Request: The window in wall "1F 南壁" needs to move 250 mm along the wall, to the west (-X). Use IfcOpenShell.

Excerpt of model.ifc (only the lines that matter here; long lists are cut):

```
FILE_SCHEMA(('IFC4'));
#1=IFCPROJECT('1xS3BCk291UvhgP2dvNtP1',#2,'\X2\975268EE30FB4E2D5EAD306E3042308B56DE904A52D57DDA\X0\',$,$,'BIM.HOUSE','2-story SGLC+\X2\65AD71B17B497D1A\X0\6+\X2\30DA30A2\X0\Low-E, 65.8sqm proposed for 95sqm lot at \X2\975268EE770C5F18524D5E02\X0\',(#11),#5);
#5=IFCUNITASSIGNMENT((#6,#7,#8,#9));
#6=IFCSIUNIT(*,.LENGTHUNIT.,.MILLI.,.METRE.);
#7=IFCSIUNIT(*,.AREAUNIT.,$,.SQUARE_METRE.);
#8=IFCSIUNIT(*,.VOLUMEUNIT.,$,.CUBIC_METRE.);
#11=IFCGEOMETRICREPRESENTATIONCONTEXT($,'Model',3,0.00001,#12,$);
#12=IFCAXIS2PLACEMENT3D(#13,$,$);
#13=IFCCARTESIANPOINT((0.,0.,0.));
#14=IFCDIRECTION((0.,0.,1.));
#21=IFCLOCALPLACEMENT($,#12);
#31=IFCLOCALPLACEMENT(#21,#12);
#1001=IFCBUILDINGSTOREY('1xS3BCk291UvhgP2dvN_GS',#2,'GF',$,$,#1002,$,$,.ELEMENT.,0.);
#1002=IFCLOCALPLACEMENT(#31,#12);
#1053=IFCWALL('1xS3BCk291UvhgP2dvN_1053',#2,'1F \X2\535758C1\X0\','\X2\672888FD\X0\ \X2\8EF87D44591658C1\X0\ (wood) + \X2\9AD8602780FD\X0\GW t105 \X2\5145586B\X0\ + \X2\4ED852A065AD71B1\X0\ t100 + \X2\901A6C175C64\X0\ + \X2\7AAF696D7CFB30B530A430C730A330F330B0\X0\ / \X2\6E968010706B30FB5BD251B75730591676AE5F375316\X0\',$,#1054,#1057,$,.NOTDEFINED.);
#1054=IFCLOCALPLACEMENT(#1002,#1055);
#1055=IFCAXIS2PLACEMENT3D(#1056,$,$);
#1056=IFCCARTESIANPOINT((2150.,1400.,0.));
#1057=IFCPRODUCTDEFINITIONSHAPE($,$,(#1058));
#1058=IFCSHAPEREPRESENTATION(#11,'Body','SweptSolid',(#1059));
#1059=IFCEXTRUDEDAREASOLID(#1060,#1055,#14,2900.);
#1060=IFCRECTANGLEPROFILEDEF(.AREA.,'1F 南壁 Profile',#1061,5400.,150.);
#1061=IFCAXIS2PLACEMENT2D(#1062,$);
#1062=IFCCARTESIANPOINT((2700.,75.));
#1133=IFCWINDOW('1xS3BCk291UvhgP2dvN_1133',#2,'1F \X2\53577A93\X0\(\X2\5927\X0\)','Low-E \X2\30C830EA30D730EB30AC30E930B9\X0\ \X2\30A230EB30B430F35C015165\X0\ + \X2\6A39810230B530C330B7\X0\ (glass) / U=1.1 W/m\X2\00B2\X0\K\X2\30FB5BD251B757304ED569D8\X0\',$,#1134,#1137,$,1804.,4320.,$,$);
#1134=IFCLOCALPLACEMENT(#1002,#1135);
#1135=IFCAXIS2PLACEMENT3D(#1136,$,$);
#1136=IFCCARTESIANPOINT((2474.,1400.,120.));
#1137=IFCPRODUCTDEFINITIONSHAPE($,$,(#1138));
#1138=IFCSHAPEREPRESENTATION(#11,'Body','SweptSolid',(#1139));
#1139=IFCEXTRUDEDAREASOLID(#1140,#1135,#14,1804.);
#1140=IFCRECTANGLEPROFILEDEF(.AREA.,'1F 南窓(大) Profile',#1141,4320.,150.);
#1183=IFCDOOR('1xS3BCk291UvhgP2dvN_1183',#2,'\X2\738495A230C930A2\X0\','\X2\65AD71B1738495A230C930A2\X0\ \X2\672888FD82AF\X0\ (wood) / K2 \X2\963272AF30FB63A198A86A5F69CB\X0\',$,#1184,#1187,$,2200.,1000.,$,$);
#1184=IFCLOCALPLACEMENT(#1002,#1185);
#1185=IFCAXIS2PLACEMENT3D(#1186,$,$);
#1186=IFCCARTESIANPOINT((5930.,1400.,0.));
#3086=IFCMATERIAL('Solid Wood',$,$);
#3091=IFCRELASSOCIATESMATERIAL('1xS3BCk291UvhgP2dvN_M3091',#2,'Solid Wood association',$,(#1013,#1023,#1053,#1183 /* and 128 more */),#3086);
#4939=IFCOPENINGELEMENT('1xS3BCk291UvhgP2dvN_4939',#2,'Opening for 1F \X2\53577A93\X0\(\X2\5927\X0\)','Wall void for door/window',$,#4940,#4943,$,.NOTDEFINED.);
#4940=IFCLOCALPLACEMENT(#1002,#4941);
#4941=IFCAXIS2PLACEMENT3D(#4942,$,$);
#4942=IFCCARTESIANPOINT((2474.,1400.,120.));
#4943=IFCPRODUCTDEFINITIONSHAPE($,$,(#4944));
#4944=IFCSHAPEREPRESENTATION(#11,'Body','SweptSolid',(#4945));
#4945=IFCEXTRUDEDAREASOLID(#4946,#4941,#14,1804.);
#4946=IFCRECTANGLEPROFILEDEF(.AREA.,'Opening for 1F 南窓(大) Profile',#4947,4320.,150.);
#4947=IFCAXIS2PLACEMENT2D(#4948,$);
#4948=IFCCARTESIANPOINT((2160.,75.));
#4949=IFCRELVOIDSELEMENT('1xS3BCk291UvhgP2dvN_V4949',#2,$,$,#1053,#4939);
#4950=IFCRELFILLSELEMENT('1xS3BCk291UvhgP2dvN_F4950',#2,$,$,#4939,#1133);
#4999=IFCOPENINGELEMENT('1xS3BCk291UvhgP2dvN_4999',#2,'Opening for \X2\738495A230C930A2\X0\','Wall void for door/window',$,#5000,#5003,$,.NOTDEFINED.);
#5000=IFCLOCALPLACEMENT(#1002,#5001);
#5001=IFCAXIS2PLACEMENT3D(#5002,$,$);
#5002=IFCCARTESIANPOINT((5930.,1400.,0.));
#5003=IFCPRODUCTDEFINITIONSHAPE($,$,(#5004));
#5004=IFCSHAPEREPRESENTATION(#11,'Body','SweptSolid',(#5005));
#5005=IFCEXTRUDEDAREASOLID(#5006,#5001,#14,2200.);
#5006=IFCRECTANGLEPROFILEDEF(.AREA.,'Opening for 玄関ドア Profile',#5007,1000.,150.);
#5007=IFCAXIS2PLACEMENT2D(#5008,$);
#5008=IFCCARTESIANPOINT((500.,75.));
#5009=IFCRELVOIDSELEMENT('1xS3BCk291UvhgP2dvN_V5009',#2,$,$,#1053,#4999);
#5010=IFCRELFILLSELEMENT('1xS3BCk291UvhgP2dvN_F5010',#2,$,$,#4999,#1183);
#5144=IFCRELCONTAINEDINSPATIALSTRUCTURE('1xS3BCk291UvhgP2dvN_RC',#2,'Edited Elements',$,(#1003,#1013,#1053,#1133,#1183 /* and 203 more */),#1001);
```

```python
import ifcopenshell
import ifcopenshell.api.geometry
import ifcopenshell.util.placement
import ifcopenshell.util.unit

model = ifcopenshell.open("model.ifc")
unit_scale = ifcopenshell.util.unit.calculate_unit_scale(model)

window = model.by_id(1133)
opening = window.FillsVoids[0].RelatingOpeningElement
wall = opening.VoidsElements[0].RelatingBuildingElement

wall_matrix = ifcopenshell.util.placement.get_local_placement(wall.ObjectPlacement)
shift = wall_matrix[:3, 0] * -0.25 / unit_scale
before = ifcopenshell.util.placement.get_local_placement(window.ObjectPlacement)[:3, 3].copy()

# The window is not placed relative to its opening, so move both.
for product in (opening, window):
    matrix = ifcopenshell.util.placement.get_local_placement(product.ObjectPlacement)
    matrix[:3, 3] += shift
    ifcopenshell.api.geometry.edit_object_placement(model, product=product, matrix=matrix, is_si=False)

after = ifcopenshell.util.placement.get_local_placement(window.ObjectPlacement)[:3, 3]
print("window moved by", (after - before).round(3) + 0.0)

model.write("model_updated.ifc")
```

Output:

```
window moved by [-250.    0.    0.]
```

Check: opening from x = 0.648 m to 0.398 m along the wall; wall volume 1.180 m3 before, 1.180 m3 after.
